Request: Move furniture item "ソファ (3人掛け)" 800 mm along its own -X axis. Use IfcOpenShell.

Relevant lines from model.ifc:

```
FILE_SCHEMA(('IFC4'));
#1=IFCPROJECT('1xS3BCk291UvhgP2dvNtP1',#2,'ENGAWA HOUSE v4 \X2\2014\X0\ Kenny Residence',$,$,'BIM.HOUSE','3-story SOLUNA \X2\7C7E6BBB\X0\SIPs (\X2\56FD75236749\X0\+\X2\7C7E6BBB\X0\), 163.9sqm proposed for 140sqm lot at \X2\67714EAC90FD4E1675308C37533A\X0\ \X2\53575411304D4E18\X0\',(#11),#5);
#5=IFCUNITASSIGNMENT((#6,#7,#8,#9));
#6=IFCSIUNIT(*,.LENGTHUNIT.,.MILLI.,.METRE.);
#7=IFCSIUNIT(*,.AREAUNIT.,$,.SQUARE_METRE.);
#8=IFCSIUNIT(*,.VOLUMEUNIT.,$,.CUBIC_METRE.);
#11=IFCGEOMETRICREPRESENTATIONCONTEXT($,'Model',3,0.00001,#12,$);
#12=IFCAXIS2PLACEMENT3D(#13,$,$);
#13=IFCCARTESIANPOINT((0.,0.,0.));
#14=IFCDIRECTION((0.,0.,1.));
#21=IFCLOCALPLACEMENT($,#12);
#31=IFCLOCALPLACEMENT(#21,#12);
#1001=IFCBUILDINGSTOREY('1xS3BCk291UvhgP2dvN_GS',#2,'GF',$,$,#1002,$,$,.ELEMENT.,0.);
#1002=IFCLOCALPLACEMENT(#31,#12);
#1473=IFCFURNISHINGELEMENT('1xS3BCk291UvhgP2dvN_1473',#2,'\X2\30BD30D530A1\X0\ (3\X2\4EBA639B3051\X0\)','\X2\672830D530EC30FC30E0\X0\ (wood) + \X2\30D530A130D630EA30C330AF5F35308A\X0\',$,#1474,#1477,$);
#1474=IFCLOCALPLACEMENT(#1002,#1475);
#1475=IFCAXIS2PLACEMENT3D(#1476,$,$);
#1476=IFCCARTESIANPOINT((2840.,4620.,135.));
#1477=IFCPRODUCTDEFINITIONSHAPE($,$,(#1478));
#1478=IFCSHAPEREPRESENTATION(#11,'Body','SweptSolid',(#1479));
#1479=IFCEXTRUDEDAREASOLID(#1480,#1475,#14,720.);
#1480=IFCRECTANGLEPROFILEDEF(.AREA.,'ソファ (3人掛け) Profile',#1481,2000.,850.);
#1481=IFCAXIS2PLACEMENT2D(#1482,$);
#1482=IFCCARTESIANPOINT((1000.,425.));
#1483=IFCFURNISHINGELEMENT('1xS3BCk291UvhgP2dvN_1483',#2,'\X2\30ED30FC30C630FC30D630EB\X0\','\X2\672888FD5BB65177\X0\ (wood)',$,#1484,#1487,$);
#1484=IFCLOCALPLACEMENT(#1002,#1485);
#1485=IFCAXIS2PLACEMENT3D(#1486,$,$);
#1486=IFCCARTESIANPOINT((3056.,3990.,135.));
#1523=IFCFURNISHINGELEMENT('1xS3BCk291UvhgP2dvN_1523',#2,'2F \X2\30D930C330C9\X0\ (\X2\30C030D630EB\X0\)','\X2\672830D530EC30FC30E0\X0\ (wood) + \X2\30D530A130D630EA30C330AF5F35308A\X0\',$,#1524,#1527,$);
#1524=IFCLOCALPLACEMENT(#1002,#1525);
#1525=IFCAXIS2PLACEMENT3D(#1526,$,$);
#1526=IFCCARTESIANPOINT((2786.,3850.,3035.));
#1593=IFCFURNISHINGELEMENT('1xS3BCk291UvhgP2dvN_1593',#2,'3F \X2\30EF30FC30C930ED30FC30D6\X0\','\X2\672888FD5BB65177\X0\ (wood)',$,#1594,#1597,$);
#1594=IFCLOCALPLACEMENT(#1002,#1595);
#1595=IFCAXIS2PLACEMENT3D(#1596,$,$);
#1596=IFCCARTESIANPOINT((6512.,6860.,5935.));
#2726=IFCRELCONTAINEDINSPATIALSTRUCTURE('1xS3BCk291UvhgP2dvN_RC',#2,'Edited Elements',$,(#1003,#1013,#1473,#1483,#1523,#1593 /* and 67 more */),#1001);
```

```python
import ifcopenshell
import ifcopenshell.api.geometry
import ifcopenshell.util.placement
import ifcopenshell.util.unit

model = ifcopenshell.open("model.ifc")
unit_scale = ifcopenshell.util.unit.calculate_unit_scale(model)

item = model.by_guid("1xS3BCk291UvhgP2dvN_1473")
matrix = ifcopenshell.util.placement.get_local_placement(item.ObjectPlacement)
matrix[:3, 3] -= matrix[:3, 0] * 0.8 / unit_scale
ifcopenshell.api.geometry.edit_object_placement(model, product=item, matrix=matrix, is_si=False)

print(ifcopenshell.util.placement.get_local_placement(item.ObjectPlacement).round(3) + 0.0)

model.write("model_updated.ifc")
```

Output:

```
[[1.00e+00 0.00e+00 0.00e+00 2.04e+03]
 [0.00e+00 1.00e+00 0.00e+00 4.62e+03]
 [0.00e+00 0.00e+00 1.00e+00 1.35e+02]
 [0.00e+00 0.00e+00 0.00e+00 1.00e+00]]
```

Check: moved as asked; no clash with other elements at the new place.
